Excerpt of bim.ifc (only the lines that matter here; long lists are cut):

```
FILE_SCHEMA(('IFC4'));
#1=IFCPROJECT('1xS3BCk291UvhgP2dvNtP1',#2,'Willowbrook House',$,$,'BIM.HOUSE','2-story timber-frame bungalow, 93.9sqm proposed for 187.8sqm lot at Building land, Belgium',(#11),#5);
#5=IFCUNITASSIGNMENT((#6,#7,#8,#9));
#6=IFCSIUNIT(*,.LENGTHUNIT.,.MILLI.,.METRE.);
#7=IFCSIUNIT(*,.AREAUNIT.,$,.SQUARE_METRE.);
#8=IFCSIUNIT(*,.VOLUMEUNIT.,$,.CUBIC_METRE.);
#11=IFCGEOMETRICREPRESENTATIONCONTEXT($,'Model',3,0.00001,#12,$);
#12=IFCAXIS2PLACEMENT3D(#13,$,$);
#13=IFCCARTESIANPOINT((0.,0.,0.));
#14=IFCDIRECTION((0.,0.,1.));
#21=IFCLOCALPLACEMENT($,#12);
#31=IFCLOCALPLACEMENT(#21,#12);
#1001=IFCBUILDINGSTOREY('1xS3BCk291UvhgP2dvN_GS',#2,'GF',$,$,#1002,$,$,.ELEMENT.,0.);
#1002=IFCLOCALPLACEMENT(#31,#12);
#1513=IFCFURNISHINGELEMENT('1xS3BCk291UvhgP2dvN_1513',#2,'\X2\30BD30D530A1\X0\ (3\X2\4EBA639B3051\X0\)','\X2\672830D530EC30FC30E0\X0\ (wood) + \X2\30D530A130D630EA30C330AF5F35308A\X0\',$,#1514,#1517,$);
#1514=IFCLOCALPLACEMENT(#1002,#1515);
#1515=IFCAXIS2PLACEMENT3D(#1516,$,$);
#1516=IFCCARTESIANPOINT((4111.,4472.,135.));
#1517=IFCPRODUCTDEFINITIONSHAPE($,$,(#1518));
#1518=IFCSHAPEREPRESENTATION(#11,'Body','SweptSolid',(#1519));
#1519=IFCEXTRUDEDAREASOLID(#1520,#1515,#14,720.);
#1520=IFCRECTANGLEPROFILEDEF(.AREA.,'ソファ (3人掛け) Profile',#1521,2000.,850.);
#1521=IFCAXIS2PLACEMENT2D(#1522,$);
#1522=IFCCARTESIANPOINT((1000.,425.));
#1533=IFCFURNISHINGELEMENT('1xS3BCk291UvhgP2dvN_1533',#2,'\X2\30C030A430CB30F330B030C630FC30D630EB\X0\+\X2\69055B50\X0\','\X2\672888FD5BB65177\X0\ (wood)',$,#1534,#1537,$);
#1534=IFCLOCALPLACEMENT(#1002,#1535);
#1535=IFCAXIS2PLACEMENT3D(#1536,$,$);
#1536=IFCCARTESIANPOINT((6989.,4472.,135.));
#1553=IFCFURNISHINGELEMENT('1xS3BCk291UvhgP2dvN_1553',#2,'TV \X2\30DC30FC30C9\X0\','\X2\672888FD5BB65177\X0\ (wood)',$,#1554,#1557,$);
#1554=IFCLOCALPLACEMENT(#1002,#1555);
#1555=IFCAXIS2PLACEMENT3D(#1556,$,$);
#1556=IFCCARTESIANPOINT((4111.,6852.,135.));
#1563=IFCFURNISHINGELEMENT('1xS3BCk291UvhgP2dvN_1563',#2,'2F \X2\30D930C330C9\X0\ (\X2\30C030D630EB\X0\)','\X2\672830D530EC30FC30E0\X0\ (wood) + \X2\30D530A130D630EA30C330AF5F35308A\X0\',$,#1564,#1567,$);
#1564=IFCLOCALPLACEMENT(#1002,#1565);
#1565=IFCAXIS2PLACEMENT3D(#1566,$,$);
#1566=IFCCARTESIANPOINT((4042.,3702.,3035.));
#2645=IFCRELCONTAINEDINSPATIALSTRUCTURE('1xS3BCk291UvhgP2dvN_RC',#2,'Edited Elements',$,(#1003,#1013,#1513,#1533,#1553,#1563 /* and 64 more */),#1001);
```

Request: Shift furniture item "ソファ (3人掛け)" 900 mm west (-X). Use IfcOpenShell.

```python
import ifcopenshell
import ifcopenshell.api.geometry
import ifcopenshell.util.placement
import ifcopenshell.util.unit

model = ifcopenshell.open("bim.ifc")
unit_scale = ifcopenshell.util.unit.calculate_unit_scale(model)

item = model.by_guid("1xS3BCk291UvhgP2dvN_1513")
matrix = ifcopenshell.util.placement.get_local_placement(item.ObjectPlacement)
matrix[0, 3] -= 0.9 / unit_scale
ifcopenshell.api.geometry.edit_object_placement(model, product=item, matrix=matrix, is_si=False)

print(ifcopenshell.util.placement.get_local_placement(item.ObjectPlacement).round(3) + 0.0)

model.write("bim_updated.ifc")
```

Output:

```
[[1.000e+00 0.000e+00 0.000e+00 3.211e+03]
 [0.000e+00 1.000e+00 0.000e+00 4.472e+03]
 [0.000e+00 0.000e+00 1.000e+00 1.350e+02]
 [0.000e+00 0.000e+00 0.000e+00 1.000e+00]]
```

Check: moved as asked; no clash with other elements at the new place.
